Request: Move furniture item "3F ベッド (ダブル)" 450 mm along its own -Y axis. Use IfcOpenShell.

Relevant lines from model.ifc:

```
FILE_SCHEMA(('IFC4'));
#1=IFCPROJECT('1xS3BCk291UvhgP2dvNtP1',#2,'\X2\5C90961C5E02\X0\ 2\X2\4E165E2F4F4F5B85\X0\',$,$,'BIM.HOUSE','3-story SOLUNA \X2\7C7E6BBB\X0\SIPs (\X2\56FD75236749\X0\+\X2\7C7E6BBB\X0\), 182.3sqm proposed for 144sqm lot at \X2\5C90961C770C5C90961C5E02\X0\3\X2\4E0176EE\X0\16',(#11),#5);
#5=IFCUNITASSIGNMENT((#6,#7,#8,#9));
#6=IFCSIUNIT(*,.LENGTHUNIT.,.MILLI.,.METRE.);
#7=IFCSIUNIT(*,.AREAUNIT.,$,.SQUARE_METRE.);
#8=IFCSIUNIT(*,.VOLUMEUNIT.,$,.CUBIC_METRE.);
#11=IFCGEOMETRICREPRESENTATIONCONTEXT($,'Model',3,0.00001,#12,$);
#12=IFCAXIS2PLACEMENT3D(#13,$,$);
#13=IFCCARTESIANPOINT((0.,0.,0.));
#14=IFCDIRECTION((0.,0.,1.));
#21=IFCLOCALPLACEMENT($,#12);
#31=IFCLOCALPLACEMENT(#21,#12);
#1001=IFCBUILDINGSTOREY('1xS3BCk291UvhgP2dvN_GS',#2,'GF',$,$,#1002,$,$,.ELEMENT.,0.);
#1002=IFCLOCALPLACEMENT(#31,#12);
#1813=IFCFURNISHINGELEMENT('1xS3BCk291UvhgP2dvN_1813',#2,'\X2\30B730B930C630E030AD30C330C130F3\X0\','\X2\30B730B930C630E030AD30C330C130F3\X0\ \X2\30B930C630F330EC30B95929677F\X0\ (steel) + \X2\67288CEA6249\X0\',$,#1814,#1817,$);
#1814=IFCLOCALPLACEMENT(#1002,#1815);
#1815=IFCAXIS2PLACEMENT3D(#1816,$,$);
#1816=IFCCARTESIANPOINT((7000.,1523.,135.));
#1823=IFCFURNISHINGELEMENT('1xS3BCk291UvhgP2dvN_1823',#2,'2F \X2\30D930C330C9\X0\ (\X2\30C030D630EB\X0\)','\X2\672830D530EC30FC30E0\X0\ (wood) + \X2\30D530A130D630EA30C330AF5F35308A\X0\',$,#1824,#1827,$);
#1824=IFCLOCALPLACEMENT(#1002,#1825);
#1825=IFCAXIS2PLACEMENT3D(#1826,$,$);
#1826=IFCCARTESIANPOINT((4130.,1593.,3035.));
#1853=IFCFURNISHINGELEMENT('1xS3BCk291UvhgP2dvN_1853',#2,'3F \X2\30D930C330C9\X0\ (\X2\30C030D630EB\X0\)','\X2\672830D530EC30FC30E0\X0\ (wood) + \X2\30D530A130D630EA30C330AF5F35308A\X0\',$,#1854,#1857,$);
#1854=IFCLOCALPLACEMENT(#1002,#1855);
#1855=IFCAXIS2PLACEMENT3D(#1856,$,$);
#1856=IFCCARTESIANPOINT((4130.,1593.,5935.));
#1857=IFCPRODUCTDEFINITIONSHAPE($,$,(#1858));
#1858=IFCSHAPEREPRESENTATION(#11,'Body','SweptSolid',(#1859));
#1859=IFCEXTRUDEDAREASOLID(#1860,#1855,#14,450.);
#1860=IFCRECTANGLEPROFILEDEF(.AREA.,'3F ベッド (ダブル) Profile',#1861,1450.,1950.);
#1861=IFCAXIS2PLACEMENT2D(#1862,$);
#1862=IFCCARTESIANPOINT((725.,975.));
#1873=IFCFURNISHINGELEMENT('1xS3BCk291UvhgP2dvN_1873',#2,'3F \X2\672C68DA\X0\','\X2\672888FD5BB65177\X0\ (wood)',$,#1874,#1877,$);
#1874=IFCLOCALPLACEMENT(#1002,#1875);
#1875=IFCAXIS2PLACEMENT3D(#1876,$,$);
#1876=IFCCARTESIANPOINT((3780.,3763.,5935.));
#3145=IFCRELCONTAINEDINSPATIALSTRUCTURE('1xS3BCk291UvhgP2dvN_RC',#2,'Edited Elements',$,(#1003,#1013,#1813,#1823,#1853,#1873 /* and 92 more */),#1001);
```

```python
import ifcopenshell
import ifcopenshell.api.geometry
import ifcopenshell.util.placement
import ifcopenshell.util.unit

model = ifcopenshell.open("model.ifc")
unit_scale = ifcopenshell.util.unit.calculate_unit_scale(model)

item = model.by_guid("1xS3BCk291UvhgP2dvN_1853")
matrix = ifcopenshell.util.placement.get_local_placement(item.ObjectPlacement)
matrix[:3, 3] -= matrix[:3, 1] * 0.45 / unit_scale
ifcopenshell.api.geometry.edit_object_placement(model, product=item, matrix=matrix, is_si=False)

print(ifcopenshell.util.placement.get_local_placement(item.ObjectPlacement).round(3) + 0.0)

model.write("model_rev.ifc")
```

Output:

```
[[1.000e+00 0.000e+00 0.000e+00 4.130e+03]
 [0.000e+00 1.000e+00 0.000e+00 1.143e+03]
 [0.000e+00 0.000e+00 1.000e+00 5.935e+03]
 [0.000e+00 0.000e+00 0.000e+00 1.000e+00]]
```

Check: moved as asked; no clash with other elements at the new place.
